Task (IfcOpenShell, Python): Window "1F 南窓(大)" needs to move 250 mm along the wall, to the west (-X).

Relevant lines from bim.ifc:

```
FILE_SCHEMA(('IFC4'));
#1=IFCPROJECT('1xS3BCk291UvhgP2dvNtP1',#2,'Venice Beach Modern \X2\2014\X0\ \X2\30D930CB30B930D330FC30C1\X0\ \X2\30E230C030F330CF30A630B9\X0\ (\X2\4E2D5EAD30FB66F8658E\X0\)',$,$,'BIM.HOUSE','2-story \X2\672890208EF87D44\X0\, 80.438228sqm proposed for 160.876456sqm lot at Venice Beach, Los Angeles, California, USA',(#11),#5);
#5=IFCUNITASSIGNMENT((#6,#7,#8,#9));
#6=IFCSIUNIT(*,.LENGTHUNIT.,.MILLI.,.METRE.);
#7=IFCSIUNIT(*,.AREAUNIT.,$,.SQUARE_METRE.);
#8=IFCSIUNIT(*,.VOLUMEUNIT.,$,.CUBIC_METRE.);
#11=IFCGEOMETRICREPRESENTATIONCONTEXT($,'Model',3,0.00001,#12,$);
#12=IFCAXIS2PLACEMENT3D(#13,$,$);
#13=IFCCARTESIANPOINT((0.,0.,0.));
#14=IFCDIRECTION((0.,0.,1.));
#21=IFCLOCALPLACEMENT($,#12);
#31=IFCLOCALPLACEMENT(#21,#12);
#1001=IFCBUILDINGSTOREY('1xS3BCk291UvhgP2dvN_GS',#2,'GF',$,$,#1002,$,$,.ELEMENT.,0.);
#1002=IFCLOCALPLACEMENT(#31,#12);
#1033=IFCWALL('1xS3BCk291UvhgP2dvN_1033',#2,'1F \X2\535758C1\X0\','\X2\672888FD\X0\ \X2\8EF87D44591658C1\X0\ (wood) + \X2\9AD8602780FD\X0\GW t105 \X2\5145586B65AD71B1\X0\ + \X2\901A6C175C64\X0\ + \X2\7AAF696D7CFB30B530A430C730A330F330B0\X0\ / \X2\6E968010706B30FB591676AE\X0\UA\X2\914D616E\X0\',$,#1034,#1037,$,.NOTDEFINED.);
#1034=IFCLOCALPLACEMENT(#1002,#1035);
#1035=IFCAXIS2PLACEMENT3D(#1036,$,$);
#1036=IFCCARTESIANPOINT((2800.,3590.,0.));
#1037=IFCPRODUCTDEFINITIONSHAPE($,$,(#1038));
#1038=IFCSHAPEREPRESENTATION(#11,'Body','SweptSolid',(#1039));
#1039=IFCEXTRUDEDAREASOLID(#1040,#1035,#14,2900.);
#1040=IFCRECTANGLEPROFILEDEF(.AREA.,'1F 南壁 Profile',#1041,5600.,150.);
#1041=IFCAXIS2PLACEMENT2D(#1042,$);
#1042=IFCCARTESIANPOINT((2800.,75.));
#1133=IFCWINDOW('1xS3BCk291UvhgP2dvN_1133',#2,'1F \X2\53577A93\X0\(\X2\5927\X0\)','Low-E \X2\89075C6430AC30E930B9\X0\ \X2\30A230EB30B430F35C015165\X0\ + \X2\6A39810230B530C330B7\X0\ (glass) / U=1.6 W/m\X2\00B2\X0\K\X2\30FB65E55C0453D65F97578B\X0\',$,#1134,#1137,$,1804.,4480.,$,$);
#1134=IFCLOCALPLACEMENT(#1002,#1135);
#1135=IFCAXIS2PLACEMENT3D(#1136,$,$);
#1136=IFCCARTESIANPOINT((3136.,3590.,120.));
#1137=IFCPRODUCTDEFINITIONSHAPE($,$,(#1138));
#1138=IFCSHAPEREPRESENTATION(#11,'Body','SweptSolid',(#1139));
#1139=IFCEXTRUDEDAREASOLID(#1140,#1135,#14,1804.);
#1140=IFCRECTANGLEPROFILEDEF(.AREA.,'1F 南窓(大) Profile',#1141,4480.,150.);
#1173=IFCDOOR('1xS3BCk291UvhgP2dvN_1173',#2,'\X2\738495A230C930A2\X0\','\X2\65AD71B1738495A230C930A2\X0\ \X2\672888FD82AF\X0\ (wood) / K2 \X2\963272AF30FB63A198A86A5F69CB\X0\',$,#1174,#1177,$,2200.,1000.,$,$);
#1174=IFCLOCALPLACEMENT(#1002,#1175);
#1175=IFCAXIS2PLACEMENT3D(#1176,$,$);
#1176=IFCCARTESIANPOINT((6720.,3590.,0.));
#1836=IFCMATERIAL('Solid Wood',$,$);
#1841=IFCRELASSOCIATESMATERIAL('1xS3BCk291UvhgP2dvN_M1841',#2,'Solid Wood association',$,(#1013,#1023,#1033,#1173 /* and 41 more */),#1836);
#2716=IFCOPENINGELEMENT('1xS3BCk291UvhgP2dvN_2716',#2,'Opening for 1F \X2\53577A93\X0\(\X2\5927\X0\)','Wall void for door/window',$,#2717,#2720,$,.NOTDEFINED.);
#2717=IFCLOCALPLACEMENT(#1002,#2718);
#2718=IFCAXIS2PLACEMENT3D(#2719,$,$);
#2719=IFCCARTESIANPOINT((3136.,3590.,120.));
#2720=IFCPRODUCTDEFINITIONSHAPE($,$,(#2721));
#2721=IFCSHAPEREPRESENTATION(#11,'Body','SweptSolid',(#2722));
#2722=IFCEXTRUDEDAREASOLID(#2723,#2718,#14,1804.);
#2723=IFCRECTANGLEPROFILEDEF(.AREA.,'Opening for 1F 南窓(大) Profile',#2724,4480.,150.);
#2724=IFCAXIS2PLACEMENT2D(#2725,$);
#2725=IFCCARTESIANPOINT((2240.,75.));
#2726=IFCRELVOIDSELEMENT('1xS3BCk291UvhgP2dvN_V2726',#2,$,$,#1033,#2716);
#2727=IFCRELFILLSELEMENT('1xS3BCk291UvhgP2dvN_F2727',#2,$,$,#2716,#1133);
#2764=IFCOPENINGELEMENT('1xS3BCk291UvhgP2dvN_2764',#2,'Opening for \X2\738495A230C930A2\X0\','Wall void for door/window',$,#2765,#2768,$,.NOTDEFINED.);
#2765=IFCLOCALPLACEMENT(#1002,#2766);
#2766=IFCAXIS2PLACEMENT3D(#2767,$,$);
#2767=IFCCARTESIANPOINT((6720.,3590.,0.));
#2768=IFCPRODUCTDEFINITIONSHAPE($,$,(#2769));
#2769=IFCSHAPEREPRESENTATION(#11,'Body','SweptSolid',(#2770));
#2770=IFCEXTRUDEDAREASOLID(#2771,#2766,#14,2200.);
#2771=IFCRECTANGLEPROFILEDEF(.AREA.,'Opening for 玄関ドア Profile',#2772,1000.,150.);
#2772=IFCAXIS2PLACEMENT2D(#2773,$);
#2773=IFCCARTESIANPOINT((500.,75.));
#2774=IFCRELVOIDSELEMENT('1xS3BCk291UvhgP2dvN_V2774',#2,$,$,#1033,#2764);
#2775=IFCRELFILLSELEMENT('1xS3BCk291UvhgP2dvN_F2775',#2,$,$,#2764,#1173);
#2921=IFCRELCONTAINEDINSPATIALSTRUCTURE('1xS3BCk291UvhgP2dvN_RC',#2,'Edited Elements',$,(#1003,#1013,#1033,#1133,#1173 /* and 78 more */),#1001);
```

```python
import ifcopenshell
import ifcopenshell.api.geometry
import ifcopenshell.util.placement

model = ifcopenshell.open("bim.ifc")

window = model.by_id(1133)
opening = window.FillsVoids[0].RelatingOpeningElement
wall = opening.VoidsElements[0].RelatingBuildingElement

wall_matrix = ifcopenshell.util.placement.get_local_placement(wall.ObjectPlacement)
shift = wall_matrix[:3, 0] * -250.0
before = ifcopenshell.util.placement.get_local_placement(window.ObjectPlacement)[:3, 3].copy()

# The window is not placed relative to its opening, so move both.
for product in (opening, window):
    matrix = ifcopenshell.util.placement.get_local_placement(product.ObjectPlacement)
    matrix[:3, 3] += shift
    ifcopenshell.api.geometry.edit_object_placement(model, product=product, matrix=matrix, is_si=False)

after = ifcopenshell.util.placement.get_local_placement(window.ObjectPlacement)[:3, 3]
print("window moved by", (after - before).round(3) + 0.0)

model.write("bim_edited.ifc")
```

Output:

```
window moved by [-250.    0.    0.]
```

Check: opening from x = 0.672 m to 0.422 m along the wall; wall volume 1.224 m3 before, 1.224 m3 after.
